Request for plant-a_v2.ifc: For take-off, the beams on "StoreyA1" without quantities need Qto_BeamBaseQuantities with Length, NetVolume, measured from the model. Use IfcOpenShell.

First a look at what the model holds.

```python
import ifcopenshell
import ifcopenshell.util.element
import ifcopenshell.util.unit

model = ifcopenshell.open("plant-a_v2.ifc")
print(model.schema)
for unit_type in ("LENGTHUNIT", "AREAUNIT", "VOLUMEUNIT"):
    print(unit_type, ifcopenshell.util.unit.calculate_unit_scale(model, unit_type))
storey = next(s for s in model.by_type("IfcBuildingStorey") if s.Name == "StoreyA1")
beams = [e for e in ifcopenshell.util.element.get_decomposition(storey) if e.is_a("IfcBeam")]
for e in sorted(beams, key=lambda e: e.id()):
    print(e.id(), e.is_a(), e.Name, list(ifcopenshell.util.element.get_psets(e, qtos_only=True)), sep=" | ")
```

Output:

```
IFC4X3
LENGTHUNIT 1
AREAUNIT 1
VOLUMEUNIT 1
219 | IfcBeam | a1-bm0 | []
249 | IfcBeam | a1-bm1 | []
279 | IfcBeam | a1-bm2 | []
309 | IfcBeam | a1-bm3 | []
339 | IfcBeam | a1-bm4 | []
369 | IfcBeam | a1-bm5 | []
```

```python
import ifcopenshell
import ifcopenshell.api.pset
import ifcopenshell.geom
import ifcopenshell.util.element
import ifcopenshell.util.shape
import ifcopenshell.util.unit

model = ifcopenshell.open("plant-a_v2.ifc")
unit_scale = ifcopenshell.util.unit.calculate_unit_scale(model)
volume_scale = ifcopenshell.util.unit.calculate_unit_scale(model, "VOLUMEUNIT")
settings = ifcopenshell.geom.settings()

storey = next(s for s in model.by_type("IfcBuildingStorey") if s.Name == "StoreyA1")
beams = [e for e in ifcopenshell.util.element.get_decomposition(storey) if e.is_a("IfcBeam")]

for e in sorted(beams, key=lambda e: e.id()):
    if ifcopenshell.util.element.get_psets(e, qtos_only=True, should_inherit=False):
        continue
    # Geometry comes back in metres, in the element's own axes.
    shape = ifcopenshell.geom.create_shape(settings, e)
    values = {
        "Length": ifcopenshell.util.shape.get_max_xyz(shape.geometry) / unit_scale,
        "NetVolume": ifcopenshell.util.shape.get_volume(shape.geometry) / volume_scale,
    }
    qto = ifcopenshell.api.pset.add_qto(model, product=e, name="Qto_BeamBaseQuantities")
    ifcopenshell.api.pset.edit_qto(model, qto=qto, properties=values)
    print(e.id(), {k: round(v, 3) for k, v in values.items()})

model.write("plant-a_v2_v2.ifc")
```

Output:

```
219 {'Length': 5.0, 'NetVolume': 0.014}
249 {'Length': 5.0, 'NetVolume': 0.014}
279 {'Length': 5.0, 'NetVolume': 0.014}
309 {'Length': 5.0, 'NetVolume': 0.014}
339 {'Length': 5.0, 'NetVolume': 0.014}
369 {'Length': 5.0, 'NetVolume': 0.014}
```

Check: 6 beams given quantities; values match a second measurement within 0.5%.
